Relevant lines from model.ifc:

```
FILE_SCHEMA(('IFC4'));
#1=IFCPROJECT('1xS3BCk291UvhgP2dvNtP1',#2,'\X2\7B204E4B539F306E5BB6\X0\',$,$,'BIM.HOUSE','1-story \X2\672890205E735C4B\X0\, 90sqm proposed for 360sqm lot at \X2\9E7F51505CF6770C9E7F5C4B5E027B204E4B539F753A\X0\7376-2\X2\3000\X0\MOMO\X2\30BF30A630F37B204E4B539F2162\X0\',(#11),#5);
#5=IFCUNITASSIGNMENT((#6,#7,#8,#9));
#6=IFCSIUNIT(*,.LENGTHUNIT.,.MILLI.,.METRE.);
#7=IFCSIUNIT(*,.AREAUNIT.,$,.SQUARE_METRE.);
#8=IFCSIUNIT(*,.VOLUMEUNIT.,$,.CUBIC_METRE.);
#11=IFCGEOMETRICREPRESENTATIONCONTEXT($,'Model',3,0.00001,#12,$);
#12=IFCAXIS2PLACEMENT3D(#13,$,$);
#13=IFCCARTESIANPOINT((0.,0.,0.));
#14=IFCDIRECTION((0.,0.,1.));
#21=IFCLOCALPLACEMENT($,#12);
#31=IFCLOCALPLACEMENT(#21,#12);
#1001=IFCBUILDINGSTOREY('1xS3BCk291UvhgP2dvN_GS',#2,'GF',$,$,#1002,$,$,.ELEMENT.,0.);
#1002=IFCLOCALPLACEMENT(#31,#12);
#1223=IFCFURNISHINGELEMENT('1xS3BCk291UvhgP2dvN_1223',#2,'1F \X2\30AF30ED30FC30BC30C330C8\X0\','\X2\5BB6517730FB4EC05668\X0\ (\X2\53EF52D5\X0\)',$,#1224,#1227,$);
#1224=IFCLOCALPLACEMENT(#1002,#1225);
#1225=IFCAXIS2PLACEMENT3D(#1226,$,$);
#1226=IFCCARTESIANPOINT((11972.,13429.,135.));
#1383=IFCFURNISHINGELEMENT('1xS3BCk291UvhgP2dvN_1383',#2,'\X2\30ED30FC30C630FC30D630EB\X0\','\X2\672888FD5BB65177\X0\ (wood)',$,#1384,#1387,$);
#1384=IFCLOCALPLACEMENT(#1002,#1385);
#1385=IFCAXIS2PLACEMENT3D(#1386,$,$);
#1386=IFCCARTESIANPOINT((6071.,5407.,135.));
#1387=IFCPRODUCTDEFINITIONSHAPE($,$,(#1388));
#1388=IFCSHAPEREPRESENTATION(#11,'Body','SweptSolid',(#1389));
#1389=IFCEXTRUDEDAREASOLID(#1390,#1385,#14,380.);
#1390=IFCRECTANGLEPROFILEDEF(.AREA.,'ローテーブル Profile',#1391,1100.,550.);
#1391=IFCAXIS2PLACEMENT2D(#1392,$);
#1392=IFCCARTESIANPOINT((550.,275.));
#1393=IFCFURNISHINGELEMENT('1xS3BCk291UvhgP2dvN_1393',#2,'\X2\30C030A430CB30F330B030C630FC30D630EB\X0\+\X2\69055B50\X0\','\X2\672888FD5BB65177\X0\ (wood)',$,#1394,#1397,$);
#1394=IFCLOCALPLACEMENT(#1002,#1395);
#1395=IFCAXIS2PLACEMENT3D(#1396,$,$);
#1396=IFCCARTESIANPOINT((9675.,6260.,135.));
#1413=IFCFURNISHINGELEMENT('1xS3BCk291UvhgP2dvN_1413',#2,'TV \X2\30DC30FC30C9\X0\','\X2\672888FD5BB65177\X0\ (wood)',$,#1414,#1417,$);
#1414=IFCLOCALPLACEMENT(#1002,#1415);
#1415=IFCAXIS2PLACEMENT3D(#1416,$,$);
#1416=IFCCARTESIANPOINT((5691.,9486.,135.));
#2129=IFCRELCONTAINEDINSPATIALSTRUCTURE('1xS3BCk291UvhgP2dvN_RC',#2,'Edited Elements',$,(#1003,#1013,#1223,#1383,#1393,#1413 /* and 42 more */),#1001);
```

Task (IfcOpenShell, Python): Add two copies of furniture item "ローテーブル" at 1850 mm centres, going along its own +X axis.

```python
import ifcopenshell
import ifcopenshell.api.geometry
import ifcopenshell.api.root
import ifcopenshell.util.element
import ifcopenshell.util.placement
import ifcopenshell.util.unit

model = ifcopenshell.open("model.ifc")
unit_scale = ifcopenshell.util.unit.calculate_unit_scale(model)


def reuse_history(source, copy):
    """copy_class also copies each property set's owner history, people and application; keep the originals."""
    for rel in copy.IsDefinedBy:
        if rel.is_a("IfcRelDefinesByProperties") and (history := rel.RelatingPropertyDefinition.OwnerHistory):
            rel.RelatingPropertyDefinition.OwnerHistory = source.OwnerHistory
            ifcopenshell.util.element.remove_deep2(model, history)


source = model.by_guid("1xS3BCk291UvhgP2dvN_1383")
base = ifcopenshell.util.placement.get_local_placement(source.ObjectPlacement)
step = base[:3, 0] * 1.85 / unit_scale

for i in range(1, 3):
    copy = ifcopenshell.api.root.copy_class(model, product=source)
    copy.Representation = ifcopenshell.util.element.copy_deep(
        model, source.Representation, exclude=["IfcGeometricRepresentationContext", "IfcRepresentationMap"]
    )
    reuse_history(source, copy)
    matrix = base.copy()
    matrix[:3, 3] += i * step
    print("added at", matrix[:3, 3].round(3) + 0.0)
    ifcopenshell.api.geometry.edit_object_placement(model, product=copy, matrix=matrix, is_si=False)

model.write("model_rev.ifc")
```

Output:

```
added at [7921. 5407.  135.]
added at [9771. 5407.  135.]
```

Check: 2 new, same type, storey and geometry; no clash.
